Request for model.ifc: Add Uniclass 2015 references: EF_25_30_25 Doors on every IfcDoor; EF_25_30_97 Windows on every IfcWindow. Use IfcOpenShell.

First a look at what the model holds.

```python
import ifcopenshell

model = ifcopenshell.open("model.ifc")
print(model.schema)
print("classifications:", [c.Name for c in model.by_type("IfcClassification")])
for ifc_class in ("IfcDoor", "IfcRoof", "IfcStair", "IfcWall", "IfcWindow"):
    print(ifc_class, len(model.by_type(ifc_class)))
```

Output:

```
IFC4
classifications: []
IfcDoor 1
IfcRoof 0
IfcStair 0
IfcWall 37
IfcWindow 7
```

```python
import ifcopenshell
import ifcopenshell.api.classification

model = ifcopenshell.open("model.ifc")

system = ifcopenshell.api.classification.add_classification(model, classification="Uniclass 2015")

codes = {
    "IfcDoor": ("EF_25_30_25", "Doors"),
    "IfcWindow": ("EF_25_30_97", "Windows"),
}
for ifc_class, (code, name) in codes.items():
    products = model.by_type(ifc_class)
    ifcopenshell.api.classification.add_reference(
        model, products=products, classification=system, identification=code, name=name
    )
    print(code, len(products))

model.write("model_rev.ifc")
```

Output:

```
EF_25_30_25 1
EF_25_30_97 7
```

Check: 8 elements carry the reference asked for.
